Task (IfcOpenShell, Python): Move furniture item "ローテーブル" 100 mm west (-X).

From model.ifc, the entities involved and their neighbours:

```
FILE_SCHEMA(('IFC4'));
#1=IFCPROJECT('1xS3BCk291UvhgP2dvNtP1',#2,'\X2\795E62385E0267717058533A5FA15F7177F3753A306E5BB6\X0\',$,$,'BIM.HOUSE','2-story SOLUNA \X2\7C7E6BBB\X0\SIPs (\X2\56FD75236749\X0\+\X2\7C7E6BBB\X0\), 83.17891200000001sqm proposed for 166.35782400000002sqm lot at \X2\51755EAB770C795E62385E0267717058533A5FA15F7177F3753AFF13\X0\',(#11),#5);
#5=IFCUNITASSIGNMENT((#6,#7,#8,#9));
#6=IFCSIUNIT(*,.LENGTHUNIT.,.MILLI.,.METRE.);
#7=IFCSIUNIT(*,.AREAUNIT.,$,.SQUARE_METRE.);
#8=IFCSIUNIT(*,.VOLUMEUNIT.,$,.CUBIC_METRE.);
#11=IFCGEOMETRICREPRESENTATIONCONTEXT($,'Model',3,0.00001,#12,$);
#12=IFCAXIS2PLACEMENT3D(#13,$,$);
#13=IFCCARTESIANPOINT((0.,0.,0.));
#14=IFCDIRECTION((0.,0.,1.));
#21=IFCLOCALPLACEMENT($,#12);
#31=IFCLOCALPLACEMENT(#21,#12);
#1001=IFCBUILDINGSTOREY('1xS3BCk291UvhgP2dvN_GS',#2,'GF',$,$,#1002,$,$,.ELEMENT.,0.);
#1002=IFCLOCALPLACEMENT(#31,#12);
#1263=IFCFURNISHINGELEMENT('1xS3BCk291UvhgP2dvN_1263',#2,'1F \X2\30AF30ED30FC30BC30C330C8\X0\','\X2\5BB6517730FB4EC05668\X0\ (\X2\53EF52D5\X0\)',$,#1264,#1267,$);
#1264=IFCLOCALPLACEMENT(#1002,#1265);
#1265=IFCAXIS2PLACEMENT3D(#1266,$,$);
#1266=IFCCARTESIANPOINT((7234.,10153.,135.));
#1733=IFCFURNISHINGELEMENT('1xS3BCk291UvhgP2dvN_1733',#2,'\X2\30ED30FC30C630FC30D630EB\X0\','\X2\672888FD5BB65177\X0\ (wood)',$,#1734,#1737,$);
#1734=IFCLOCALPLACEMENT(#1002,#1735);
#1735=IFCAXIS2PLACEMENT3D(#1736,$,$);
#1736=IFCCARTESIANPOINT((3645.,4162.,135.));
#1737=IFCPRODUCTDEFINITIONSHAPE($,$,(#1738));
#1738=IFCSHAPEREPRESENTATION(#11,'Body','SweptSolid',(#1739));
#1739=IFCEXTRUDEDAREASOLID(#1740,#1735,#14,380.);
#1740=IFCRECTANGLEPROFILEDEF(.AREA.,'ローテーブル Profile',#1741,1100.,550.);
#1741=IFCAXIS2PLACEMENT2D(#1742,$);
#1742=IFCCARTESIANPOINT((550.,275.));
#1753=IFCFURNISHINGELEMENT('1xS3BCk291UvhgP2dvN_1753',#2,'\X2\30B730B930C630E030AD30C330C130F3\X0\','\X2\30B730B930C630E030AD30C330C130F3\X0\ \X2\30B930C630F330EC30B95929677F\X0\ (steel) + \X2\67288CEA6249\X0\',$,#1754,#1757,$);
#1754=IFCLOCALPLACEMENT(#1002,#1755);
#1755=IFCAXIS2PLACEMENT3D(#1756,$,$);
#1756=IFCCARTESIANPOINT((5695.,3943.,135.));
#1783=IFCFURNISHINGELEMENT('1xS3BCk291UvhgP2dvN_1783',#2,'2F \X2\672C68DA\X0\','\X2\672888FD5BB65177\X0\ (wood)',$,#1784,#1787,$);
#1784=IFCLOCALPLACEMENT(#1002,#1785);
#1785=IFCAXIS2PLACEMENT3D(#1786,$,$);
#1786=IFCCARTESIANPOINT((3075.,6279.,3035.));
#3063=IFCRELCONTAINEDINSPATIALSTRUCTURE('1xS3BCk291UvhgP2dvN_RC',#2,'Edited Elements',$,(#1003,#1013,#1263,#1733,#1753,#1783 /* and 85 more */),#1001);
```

```python
import ifcopenshell
import ifcopenshell.api.geometry
import ifcopenshell.util.placement

model = ifcopenshell.open("model.ifc")

item = model.by_guid("1xS3BCk291UvhgP2dvN_1733")
matrix = ifcopenshell.util.placement.get_local_placement(item.ObjectPlacement)
matrix[0, 3] -= 100.0
ifcopenshell.api.geometry.edit_object_placement(model, product=item, matrix=matrix, is_si=False)

print(ifcopenshell.util.placement.get_local_placement(item.ObjectPlacement).round(3) + 0.0)

model.write("model_edited.ifc")
```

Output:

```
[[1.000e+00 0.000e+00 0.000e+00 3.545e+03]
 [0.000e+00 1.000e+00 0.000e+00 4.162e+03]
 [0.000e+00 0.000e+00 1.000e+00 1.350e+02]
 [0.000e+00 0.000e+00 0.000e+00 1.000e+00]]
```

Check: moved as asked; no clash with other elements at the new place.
